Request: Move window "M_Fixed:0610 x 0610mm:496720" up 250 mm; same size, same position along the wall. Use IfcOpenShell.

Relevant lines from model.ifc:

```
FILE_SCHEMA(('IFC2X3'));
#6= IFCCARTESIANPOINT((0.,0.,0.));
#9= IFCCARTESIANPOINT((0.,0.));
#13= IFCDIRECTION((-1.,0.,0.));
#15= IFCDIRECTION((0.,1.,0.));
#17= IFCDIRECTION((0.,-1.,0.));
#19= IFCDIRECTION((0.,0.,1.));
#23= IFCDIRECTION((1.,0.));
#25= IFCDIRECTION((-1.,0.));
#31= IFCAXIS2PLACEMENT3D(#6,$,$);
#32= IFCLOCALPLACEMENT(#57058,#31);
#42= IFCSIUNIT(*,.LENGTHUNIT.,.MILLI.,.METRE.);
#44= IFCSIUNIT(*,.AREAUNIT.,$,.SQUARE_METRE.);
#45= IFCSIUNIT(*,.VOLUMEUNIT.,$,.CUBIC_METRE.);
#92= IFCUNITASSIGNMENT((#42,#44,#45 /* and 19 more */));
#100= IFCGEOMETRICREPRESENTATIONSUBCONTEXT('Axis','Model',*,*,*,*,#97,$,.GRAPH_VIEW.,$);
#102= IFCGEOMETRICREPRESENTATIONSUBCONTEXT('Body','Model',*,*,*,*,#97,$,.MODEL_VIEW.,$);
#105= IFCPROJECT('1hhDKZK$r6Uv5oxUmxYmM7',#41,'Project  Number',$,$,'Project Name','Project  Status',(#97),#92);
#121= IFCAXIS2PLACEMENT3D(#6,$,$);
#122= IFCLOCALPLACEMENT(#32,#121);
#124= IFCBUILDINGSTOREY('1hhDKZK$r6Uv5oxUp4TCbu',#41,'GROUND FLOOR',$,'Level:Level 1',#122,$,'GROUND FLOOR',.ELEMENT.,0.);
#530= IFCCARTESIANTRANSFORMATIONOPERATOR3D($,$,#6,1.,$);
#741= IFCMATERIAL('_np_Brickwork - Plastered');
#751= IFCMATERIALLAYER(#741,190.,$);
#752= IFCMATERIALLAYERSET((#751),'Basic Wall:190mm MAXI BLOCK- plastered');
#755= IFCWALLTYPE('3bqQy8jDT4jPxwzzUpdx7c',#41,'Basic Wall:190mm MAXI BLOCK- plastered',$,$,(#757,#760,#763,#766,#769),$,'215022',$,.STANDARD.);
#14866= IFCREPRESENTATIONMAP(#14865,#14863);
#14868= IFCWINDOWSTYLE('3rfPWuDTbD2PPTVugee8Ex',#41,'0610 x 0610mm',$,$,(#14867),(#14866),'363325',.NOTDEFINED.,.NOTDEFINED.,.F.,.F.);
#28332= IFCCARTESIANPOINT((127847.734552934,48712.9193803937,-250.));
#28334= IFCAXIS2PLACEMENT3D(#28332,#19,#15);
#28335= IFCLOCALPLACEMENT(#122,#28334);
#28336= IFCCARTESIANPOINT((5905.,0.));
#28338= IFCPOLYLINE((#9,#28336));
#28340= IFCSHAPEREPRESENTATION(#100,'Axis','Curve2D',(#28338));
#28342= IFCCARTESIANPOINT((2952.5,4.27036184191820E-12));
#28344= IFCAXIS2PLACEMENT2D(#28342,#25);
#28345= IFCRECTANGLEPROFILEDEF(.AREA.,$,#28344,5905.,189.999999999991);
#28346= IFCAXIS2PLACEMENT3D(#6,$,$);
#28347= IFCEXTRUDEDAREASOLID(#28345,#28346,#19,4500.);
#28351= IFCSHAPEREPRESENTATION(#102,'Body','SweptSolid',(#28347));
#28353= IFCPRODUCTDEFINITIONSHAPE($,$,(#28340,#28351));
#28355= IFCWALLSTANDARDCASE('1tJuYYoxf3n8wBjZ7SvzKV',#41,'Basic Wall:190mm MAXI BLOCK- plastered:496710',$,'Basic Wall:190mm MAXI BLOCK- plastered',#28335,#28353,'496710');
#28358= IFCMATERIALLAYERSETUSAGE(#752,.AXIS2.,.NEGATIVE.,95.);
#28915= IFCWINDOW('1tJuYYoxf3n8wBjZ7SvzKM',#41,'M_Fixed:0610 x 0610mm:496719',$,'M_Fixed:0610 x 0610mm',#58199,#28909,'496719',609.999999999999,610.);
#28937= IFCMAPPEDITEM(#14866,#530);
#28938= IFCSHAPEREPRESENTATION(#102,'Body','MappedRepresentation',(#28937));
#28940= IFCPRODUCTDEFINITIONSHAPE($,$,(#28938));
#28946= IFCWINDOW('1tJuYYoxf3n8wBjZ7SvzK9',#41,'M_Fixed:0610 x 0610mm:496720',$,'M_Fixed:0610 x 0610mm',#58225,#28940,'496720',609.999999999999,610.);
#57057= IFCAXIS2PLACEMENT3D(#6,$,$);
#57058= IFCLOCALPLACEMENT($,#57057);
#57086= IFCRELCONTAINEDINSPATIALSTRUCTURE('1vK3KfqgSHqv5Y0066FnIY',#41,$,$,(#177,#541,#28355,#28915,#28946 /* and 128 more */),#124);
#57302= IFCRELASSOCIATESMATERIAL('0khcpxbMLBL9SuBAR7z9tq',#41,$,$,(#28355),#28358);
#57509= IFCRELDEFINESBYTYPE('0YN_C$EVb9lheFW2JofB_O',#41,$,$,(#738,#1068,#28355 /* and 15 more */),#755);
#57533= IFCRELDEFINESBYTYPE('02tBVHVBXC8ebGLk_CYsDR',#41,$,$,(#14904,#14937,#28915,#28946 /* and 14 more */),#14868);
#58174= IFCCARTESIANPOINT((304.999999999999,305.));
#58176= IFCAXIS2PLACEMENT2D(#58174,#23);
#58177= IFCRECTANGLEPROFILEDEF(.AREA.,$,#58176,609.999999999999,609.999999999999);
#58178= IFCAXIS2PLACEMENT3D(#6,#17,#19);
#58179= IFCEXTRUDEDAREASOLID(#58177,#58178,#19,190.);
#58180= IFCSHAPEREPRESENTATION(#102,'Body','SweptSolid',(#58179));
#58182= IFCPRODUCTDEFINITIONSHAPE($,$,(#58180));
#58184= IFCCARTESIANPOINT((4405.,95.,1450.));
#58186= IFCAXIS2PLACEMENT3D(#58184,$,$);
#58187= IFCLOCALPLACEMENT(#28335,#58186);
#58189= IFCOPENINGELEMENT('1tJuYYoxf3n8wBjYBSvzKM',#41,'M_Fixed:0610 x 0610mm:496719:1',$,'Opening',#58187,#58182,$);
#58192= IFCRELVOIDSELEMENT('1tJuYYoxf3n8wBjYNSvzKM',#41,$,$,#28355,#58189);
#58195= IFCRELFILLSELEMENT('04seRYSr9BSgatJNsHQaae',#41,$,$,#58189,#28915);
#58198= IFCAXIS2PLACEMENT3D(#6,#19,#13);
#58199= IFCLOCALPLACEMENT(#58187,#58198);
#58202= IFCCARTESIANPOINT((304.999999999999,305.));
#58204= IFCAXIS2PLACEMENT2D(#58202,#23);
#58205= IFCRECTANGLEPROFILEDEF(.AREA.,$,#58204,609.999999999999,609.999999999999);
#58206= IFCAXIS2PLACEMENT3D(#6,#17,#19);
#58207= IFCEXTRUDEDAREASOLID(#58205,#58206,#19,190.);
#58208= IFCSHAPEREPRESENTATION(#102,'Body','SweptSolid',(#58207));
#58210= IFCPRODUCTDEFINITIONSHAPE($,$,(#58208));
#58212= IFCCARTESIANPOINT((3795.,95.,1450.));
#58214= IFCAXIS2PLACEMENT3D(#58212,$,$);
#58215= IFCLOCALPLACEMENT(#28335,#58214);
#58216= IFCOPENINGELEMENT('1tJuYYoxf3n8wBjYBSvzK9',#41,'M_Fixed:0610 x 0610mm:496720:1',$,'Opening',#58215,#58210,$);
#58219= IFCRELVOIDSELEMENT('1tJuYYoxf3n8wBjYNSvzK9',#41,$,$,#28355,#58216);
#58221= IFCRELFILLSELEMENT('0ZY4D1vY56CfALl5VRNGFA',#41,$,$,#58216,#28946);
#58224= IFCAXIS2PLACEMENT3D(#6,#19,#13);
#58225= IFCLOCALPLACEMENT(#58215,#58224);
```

```python
import numpy as np
import ifcopenshell
import ifcopenshell.api.geometry
import ifcopenshell.util.placement
import ifcopenshell.util.unit

model = ifcopenshell.open("model.ifc")
unit_scale = ifcopenshell.util.unit.calculate_unit_scale(model)

window = model.by_guid("1tJuYYoxf3n8wBjZ7SvzK9")
opening = window.FillsVoids[0].RelatingOpeningElement
dz = 250.0

shift = np.array([0.0, 0.0, dz])
# The window is placed relative to its opening, so it follows when the opening moves.
matrix = ifcopenshell.util.placement.get_local_placement(opening.ObjectPlacement)
matrix[:3, 3] += shift
ifcopenshell.api.geometry.edit_object_placement(
    model, product=opening, matrix=matrix, is_si=False, should_transform_children=True
)

print(f"moved by {dz * unit_scale:+.3f} m")

model.write("model_v2.ifc")
```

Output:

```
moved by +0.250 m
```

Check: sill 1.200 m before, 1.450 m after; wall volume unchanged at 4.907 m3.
